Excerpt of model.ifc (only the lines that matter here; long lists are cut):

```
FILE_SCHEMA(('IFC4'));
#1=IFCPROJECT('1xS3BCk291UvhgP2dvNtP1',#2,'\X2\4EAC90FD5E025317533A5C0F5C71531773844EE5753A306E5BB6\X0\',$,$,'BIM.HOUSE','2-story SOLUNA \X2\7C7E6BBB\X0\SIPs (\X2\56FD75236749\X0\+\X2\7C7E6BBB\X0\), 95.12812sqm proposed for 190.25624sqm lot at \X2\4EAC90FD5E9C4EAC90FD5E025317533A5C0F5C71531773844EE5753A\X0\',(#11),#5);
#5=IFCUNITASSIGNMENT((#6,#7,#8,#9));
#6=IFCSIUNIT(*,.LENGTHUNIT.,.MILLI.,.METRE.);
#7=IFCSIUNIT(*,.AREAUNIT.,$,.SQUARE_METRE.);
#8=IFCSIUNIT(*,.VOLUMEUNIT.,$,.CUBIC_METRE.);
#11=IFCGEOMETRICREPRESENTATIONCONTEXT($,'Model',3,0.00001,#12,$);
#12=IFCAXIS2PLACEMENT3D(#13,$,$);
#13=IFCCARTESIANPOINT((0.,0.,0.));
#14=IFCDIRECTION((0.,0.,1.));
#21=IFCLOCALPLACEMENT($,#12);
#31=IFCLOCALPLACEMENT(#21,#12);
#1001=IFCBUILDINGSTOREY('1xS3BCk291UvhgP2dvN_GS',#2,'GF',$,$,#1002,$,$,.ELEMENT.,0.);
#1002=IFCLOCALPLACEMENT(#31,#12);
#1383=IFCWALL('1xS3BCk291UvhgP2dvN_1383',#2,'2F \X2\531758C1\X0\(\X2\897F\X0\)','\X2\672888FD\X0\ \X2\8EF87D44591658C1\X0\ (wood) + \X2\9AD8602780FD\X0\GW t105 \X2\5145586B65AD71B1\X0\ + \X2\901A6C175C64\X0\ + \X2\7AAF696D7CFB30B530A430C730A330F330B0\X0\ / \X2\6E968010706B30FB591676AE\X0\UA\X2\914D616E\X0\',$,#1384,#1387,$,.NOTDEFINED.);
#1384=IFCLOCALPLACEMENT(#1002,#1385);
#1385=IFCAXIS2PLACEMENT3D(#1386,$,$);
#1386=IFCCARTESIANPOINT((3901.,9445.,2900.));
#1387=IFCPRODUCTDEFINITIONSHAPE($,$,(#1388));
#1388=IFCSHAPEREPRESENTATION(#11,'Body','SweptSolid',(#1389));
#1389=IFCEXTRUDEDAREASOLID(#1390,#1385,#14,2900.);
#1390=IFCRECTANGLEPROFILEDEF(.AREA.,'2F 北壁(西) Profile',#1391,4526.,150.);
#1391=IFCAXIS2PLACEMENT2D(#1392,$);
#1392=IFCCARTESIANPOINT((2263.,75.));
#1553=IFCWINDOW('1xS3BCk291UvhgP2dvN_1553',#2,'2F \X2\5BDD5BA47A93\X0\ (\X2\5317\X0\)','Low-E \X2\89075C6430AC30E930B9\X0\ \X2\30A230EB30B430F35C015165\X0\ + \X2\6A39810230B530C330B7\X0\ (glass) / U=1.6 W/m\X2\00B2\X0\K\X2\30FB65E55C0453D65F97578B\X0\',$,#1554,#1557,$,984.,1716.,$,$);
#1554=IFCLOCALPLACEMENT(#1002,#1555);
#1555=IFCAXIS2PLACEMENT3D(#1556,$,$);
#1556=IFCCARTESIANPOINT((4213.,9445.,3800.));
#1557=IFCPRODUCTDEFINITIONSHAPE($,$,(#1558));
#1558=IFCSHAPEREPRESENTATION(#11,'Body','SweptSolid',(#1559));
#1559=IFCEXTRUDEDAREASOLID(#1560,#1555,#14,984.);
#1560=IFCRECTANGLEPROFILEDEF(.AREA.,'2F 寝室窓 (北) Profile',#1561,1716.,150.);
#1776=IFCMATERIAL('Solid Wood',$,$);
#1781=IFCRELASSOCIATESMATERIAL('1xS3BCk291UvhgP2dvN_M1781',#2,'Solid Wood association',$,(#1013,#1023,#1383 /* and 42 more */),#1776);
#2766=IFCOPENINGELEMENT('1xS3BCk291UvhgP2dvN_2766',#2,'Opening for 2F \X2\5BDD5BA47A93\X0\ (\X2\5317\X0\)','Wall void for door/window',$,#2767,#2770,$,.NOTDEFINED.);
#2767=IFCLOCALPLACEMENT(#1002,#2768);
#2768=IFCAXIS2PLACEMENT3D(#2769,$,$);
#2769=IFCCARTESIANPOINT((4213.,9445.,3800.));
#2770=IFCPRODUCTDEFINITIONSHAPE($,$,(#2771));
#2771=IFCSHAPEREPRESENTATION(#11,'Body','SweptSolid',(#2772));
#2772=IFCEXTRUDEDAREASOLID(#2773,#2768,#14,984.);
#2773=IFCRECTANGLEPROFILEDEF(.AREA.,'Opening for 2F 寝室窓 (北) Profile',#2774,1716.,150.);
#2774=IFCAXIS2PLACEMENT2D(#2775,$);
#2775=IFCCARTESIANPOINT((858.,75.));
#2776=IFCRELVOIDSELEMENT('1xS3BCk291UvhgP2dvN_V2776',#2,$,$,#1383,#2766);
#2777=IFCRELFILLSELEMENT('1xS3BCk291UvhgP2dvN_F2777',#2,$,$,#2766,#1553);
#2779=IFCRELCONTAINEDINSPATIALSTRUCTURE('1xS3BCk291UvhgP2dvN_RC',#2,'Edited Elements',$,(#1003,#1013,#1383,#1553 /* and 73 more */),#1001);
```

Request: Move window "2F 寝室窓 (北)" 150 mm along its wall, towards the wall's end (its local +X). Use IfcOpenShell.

```python
import ifcopenshell
import ifcopenshell.api.geometry
import ifcopenshell.util.placement

model = ifcopenshell.open("model.ifc")

window = model.by_guid("1xS3BCk291UvhgP2dvN_1553")
opening = window.FillsVoids[0].RelatingOpeningElement
wall = opening.VoidsElements[0].RelatingBuildingElement

wall_matrix = ifcopenshell.util.placement.get_local_placement(wall.ObjectPlacement)
shift = wall_matrix[:3, 0] * 150.0
before = ifcopenshell.util.placement.get_local_placement(window.ObjectPlacement)[:3, 3].copy()

# The window is not placed relative to its opening, so move both.
for product in (opening, window):
    matrix = ifcopenshell.util.placement.get_local_placement(product.ObjectPlacement)
    matrix[:3, 3] += shift
    ifcopenshell.api.geometry.edit_object_placement(model, product=product, matrix=matrix, is_si=False)

after = ifcopenshell.util.placement.get_local_placement(window.ObjectPlacement)[:3, 3]
print("window moved by", (after - before).round(3) + 0.0)

model.write("model-out.ifc")
```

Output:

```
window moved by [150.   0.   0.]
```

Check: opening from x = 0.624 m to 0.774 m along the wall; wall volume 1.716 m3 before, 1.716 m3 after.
